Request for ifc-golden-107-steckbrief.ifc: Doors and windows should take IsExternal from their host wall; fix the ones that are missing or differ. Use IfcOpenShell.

First a look at what the model holds.

```python
import ifcopenshell
import ifcopenshell.util.element

model = ifcopenshell.open("ifc-golden-107-steckbrief.ifc")
print(model.schema)
seen = {}
for e in model.by_type("IfcDoor") + model.by_type("IfcWindow"):
    if not e.FillsVoids:
        continue
    host = e.FillsVoids[0].RelatingOpeningElement.VoidsElements[0].RelatingBuildingElement
    own = ifcopenshell.util.element.get_pset(e, f"Pset_{e.is_a()[3:].removesuffix('StandardCase')}Common", "IsExternal")
    wall = ifcopenshell.util.element.get_pset(host, "Pset_WallCommon", "IsExternal")
    seen[e.is_a(), own, wall] = seen.get((e.is_a(), own, wall), 0) + 1
for (cls, own, wall), count in sorted(seen.items(), key=str):
    print(count, cls, "IsExternal:", own, "| host wall:", wall)
```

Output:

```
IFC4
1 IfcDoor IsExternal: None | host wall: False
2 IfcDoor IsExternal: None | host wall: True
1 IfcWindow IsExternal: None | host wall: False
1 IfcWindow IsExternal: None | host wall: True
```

```python
import ifcopenshell
import ifcopenshell.api.pset
import ifcopenshell.util.element

model = ifcopenshell.open("ifc-golden-107-steckbrief.ifc")

count = 0
for ifc_class, pset_name in (("IfcDoor", "Pset_DoorCommon"), ("IfcWindow", "Pset_WindowCommon")):
    for e in model.by_type(ifc_class):
        if not e.FillsVoids:
            continue
        host = e.FillsVoids[0].RelatingOpeningElement.VoidsElements[0].RelatingBuildingElement
        external = ifcopenshell.util.element.get_pset(host, "Pset_WallCommon", "IsExternal")
        if external is None or ifcopenshell.util.element.get_pset(e, pset_name, "IsExternal") == external:
            continue
        pset = ifcopenshell.api.pset.add_pset(model, product=e, name=pset_name)
        ifcopenshell.api.pset.edit_pset(model, pset=pset, properties={"IsExternal": external})
        count += 1

print(count, "updated")

model.write("ifc-golden-107-steckbrief-out.ifc")
```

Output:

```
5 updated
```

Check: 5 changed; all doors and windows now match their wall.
